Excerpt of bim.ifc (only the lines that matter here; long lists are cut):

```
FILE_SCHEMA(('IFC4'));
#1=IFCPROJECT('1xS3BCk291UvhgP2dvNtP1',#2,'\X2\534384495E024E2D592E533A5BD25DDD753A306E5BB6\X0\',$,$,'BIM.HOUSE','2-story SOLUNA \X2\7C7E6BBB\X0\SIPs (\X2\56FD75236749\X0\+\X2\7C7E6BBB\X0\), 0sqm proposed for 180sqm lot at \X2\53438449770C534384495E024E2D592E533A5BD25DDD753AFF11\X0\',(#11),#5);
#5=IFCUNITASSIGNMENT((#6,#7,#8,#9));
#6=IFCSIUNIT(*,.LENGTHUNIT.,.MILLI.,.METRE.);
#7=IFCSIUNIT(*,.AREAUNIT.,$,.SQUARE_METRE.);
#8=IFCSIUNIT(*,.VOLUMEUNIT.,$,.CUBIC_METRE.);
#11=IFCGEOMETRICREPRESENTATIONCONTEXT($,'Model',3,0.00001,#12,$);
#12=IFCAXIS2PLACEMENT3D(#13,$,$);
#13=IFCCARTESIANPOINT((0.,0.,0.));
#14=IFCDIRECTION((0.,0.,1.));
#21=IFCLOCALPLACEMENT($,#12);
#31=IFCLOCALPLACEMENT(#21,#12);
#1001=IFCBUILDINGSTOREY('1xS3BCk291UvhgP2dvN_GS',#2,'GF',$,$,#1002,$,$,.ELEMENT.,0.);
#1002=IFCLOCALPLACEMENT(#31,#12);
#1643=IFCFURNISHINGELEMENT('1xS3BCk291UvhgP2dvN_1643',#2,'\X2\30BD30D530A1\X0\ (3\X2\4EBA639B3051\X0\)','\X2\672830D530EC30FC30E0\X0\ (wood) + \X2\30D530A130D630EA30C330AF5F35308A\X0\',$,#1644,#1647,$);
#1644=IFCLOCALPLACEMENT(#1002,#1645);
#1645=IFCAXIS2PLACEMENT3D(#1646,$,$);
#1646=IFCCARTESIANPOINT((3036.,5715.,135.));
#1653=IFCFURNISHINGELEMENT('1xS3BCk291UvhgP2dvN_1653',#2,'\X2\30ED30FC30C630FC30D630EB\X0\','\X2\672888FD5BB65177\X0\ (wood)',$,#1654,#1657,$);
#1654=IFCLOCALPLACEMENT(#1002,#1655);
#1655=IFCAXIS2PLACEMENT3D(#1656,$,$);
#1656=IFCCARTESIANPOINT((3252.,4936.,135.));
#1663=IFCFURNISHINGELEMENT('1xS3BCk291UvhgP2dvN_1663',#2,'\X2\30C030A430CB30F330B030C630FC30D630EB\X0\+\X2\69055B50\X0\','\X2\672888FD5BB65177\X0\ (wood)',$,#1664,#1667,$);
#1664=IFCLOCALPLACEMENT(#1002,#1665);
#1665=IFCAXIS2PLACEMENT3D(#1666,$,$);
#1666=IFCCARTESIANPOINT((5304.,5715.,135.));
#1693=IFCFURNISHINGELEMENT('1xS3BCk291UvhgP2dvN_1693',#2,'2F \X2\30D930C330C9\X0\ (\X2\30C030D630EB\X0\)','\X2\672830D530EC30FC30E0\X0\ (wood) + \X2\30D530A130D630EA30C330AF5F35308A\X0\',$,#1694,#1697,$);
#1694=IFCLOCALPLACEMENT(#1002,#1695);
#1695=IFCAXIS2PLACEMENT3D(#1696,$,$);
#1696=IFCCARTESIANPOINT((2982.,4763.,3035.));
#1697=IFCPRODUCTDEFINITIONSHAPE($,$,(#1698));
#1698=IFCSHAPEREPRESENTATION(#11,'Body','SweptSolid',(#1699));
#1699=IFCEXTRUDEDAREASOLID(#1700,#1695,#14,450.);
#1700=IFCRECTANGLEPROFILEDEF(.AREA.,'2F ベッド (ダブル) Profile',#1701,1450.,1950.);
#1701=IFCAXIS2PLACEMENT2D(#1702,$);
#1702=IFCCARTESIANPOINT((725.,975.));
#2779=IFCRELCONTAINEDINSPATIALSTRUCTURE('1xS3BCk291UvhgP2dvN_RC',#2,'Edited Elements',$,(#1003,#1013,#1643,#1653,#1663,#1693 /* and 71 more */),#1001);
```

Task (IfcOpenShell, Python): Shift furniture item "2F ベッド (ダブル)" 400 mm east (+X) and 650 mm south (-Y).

```python
import ifcopenshell
import ifcopenshell.api.geometry
import ifcopenshell.util.placement

model = ifcopenshell.open("bim.ifc")

item = model.by_guid("1xS3BCk291UvhgP2dvN_1693")
matrix = ifcopenshell.util.placement.get_local_placement(item.ObjectPlacement)
matrix[0, 3] += 400.0
matrix[1, 3] -= 650.0
ifcopenshell.api.geometry.edit_object_placement(model, product=item, matrix=matrix, is_si=False)

print(ifcopenshell.util.placement.get_local_placement(item.ObjectPlacement).round(3) + 0.0)

model.write("bim_updated.ifc")
```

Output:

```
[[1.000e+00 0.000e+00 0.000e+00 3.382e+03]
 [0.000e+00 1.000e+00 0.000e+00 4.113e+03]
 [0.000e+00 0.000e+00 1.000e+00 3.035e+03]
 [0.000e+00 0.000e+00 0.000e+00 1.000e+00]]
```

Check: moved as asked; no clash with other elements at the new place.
